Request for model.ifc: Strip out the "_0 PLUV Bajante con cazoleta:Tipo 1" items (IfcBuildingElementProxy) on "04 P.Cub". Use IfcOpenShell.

First a look at what the model holds.

```python
import ifcopenshell
import ifcopenshell.util.element

model = ifcopenshell.open("model.ifc")
print(model.schema)
storey = next(s for s in model.by_type("IfcBuildingStorey") if s.Name == "04 P.Cub")
proxies = [e for e in ifcopenshell.util.element.get_decomposition(storey) if e.is_a("IfcBuildingElementProxy")]
seen = {}
for e in proxies:
    element_type = ifcopenshell.util.element.get_type(e)
    name = element_type.Name if element_type not in (None, e) else None
    seen[name] = seen.get(name, 0) + 1
for name, count in sorted(seen.items(), key=str):
    print(count, "x", name)
```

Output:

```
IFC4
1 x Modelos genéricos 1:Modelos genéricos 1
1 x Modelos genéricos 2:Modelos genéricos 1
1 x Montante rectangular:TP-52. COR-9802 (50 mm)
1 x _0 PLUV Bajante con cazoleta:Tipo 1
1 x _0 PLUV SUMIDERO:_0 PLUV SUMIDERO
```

```python
import ifcopenshell
import ifcopenshell.api.root
import ifcopenshell.util.element

model = ifcopenshell.open("model.ifc")

storey = next(s for s in model.by_type("IfcBuildingStorey") if s.Name == "04 P.Cub")
proxies = [e for e in ifcopenshell.util.element.get_decomposition(storey) if e.is_a("IfcBuildingElementProxy")]
targets = [e for e in proxies if (t := ifcopenshell.util.element.get_type(e)) not in (None, e) and t.Name == "_0 PLUV Bajante con cazoleta:Tipo 1"]

for e in targets:
    ifcopenshell.api.root.remove_product(model, product=e)
print(len(targets), "removed")

model.write("model_rev.ifc")
```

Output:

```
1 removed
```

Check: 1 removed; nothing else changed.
